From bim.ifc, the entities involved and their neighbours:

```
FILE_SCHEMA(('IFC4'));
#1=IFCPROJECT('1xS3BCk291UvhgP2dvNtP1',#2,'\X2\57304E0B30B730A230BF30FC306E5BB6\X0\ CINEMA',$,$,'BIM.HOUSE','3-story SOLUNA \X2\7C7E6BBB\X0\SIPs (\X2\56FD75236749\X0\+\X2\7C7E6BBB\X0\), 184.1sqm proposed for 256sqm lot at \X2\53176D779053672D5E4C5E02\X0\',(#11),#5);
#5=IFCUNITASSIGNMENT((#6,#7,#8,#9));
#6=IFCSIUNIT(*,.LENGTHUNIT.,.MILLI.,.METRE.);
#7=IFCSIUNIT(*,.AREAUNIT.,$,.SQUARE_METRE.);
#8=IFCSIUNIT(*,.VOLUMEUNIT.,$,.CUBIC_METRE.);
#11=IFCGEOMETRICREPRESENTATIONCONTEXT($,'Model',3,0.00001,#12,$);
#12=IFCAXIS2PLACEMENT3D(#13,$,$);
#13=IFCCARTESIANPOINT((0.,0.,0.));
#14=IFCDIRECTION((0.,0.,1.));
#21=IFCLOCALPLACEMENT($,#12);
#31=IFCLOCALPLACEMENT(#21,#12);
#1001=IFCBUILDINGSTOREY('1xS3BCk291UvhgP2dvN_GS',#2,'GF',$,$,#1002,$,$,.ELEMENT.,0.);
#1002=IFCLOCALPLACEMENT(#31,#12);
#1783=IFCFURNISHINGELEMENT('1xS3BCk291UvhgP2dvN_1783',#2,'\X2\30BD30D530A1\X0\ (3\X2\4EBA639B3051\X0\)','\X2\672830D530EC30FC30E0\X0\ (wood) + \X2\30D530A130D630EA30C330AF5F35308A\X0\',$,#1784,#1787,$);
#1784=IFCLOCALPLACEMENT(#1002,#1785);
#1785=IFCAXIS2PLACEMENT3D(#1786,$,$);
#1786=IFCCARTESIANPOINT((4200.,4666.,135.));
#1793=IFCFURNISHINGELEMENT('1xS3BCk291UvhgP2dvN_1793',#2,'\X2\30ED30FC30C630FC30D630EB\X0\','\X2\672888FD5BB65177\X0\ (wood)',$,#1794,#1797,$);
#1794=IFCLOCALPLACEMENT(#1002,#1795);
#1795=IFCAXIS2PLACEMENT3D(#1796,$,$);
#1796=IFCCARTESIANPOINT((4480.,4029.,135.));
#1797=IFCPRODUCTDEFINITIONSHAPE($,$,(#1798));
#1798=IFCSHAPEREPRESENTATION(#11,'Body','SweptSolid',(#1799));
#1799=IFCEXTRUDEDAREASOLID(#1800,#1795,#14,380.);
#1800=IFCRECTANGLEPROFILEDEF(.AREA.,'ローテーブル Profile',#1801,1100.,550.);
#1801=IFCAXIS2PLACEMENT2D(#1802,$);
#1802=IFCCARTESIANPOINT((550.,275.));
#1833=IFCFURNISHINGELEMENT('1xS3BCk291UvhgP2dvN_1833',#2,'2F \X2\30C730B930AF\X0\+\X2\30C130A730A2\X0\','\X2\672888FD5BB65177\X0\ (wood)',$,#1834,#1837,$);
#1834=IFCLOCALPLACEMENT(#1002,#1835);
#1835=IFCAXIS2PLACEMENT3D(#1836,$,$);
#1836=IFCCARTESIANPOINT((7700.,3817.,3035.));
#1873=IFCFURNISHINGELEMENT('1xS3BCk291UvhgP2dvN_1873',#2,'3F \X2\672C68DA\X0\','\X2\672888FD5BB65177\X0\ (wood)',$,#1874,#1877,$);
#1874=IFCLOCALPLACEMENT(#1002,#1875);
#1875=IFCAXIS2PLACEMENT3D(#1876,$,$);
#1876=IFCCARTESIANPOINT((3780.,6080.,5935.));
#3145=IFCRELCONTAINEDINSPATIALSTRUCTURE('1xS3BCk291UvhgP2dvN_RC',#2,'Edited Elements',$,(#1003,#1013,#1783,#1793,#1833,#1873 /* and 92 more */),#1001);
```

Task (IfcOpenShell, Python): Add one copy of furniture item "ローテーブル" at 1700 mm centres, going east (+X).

```python
import numpy as np
import ifcopenshell
import ifcopenshell.api.geometry
import ifcopenshell.api.root
import ifcopenshell.util.element
import ifcopenshell.util.placement

model = ifcopenshell.open("bim.ifc")


def reuse_history(source, copy):
    """copy_class also copies each property set's owner history, people and application; keep the originals."""
    for rel in copy.IsDefinedBy:
        if rel.is_a("IfcRelDefinesByProperties") and (history := rel.RelatingPropertyDefinition.OwnerHistory):
            rel.RelatingPropertyDefinition.OwnerHistory = source.OwnerHistory
            ifcopenshell.util.element.remove_deep2(model, history)


source = model.by_guid("1xS3BCk291UvhgP2dvN_1793")
base = ifcopenshell.util.placement.get_local_placement(source.ObjectPlacement)
step = np.array([1.0, 0.0, 0.0]) * 1700.0

for i in range(1, 2):
    copy = ifcopenshell.api.root.copy_class(model, product=source)
    copy.Representation = ifcopenshell.util.element.copy_deep(
        model, source.Representation, exclude=["IfcGeometricRepresentationContext", "IfcRepresentationMap"]
    )
    reuse_history(source, copy)
    matrix = base.copy()
    matrix[:3, 3] += i * step
    print("added at", matrix[:3, 3].round(3) + 0.0)
    ifcopenshell.api.geometry.edit_object_placement(model, product=copy, matrix=matrix, is_si=False)

model.write("bim-out.ifc")
```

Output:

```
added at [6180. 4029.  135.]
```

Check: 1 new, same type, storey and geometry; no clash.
